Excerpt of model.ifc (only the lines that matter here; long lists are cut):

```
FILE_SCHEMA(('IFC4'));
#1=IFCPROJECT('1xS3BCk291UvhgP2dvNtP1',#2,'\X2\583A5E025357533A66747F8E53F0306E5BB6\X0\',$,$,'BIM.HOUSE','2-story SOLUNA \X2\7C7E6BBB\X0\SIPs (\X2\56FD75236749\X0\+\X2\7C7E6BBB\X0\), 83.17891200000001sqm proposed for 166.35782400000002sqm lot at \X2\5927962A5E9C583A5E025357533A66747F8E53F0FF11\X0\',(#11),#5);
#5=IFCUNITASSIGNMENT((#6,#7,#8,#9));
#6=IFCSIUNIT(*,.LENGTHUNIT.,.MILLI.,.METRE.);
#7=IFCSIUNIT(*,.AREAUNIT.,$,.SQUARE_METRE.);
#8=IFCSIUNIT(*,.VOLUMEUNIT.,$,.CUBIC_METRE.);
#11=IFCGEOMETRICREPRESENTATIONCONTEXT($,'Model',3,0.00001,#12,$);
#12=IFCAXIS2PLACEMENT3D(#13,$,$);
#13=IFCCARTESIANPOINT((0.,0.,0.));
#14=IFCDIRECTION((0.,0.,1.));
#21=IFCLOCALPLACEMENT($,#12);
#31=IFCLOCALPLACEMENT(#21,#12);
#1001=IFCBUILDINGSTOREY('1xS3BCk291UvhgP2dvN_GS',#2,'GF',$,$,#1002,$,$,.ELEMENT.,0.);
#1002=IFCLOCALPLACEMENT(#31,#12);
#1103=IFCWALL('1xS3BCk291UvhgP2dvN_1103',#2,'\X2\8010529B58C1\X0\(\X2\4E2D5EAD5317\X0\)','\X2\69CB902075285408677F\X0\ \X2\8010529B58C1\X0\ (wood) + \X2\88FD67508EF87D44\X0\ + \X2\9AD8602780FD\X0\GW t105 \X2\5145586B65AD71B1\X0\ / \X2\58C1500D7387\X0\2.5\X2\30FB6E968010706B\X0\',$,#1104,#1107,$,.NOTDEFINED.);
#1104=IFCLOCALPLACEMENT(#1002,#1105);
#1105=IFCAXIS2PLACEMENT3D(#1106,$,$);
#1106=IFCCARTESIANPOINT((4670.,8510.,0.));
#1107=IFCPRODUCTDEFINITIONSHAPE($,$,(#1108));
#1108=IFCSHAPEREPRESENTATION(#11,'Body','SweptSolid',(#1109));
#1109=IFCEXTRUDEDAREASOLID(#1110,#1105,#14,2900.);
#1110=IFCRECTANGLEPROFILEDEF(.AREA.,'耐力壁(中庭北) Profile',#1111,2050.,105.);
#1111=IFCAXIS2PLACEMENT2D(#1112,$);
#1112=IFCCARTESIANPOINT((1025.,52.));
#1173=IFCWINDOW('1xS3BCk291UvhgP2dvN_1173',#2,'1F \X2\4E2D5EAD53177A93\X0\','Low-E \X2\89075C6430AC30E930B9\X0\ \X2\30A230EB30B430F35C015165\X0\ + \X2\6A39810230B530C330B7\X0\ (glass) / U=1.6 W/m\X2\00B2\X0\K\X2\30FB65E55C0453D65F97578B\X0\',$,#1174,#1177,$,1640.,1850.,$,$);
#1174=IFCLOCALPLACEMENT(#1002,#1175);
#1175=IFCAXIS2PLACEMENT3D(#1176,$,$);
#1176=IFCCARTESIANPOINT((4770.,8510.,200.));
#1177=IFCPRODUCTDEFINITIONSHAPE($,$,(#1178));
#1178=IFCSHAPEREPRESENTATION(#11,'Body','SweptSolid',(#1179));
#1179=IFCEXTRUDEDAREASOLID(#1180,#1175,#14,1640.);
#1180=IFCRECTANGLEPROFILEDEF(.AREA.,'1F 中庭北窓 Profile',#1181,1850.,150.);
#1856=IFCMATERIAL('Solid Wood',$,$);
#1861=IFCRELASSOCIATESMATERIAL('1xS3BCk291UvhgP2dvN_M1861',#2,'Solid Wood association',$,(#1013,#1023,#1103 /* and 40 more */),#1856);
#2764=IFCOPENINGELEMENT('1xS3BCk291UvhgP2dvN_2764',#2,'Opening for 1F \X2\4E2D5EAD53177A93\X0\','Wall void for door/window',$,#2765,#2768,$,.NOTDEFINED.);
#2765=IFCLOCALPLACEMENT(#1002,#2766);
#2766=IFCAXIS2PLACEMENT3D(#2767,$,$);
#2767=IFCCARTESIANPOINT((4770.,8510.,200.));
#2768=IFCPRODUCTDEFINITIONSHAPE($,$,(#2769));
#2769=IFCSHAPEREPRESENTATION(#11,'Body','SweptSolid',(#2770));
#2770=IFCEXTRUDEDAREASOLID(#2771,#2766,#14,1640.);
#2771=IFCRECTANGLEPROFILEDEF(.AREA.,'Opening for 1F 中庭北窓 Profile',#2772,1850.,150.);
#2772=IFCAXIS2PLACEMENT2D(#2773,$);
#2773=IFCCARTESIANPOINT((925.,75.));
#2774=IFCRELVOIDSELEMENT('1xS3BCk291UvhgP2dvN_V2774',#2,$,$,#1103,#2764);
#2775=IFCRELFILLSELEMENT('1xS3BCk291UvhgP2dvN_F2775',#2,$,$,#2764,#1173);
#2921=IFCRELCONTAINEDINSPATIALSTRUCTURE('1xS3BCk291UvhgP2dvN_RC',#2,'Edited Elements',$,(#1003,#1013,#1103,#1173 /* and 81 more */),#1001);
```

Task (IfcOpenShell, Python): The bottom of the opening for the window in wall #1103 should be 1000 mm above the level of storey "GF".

```python
import numpy as np
import ifcopenshell
import ifcopenshell.api.geometry
import ifcopenshell.geom
import ifcopenshell.util.element
import ifcopenshell.util.placement
import ifcopenshell.util.shape
import ifcopenshell.util.unit

model = ifcopenshell.open("model.ifc")
unit_scale = ifcopenshell.util.unit.calculate_unit_scale(model)

window = model.by_id(1173)
opening = window.FillsVoids[0].RelatingOpeningElement
storey = ifcopenshell.util.element.get_container(window, ifc_class="IfcBuildingStorey")
level = ifcopenshell.util.placement.get_local_placement(storey.ObjectPlacement)[2, 3]

# The opening's origin need not be at the sill, so measure its lowest point.
shape = ifcopenshell.geom.create_shape(ifcopenshell.geom.settings(), opening)
bottom = ifcopenshell.util.shape.get_shape_bottom_elevation(shape, shape.geometry) / unit_scale
dz = level + 1 / unit_scale - bottom

shift = np.array([0.0, 0.0, dz])
# The window is not placed relative to its opening, so move both.
for product in (opening, window):
    matrix = ifcopenshell.util.placement.get_local_placement(product.ObjectPlacement)
    matrix[:3, 3] += shift
    ifcopenshell.api.geometry.edit_object_placement(model, product=product, matrix=matrix, is_si=False)

print(f"moved by {dz * unit_scale:+.3f} m")

model.write("model_v2.ifc")
```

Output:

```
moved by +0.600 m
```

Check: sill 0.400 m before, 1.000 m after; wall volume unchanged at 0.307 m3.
